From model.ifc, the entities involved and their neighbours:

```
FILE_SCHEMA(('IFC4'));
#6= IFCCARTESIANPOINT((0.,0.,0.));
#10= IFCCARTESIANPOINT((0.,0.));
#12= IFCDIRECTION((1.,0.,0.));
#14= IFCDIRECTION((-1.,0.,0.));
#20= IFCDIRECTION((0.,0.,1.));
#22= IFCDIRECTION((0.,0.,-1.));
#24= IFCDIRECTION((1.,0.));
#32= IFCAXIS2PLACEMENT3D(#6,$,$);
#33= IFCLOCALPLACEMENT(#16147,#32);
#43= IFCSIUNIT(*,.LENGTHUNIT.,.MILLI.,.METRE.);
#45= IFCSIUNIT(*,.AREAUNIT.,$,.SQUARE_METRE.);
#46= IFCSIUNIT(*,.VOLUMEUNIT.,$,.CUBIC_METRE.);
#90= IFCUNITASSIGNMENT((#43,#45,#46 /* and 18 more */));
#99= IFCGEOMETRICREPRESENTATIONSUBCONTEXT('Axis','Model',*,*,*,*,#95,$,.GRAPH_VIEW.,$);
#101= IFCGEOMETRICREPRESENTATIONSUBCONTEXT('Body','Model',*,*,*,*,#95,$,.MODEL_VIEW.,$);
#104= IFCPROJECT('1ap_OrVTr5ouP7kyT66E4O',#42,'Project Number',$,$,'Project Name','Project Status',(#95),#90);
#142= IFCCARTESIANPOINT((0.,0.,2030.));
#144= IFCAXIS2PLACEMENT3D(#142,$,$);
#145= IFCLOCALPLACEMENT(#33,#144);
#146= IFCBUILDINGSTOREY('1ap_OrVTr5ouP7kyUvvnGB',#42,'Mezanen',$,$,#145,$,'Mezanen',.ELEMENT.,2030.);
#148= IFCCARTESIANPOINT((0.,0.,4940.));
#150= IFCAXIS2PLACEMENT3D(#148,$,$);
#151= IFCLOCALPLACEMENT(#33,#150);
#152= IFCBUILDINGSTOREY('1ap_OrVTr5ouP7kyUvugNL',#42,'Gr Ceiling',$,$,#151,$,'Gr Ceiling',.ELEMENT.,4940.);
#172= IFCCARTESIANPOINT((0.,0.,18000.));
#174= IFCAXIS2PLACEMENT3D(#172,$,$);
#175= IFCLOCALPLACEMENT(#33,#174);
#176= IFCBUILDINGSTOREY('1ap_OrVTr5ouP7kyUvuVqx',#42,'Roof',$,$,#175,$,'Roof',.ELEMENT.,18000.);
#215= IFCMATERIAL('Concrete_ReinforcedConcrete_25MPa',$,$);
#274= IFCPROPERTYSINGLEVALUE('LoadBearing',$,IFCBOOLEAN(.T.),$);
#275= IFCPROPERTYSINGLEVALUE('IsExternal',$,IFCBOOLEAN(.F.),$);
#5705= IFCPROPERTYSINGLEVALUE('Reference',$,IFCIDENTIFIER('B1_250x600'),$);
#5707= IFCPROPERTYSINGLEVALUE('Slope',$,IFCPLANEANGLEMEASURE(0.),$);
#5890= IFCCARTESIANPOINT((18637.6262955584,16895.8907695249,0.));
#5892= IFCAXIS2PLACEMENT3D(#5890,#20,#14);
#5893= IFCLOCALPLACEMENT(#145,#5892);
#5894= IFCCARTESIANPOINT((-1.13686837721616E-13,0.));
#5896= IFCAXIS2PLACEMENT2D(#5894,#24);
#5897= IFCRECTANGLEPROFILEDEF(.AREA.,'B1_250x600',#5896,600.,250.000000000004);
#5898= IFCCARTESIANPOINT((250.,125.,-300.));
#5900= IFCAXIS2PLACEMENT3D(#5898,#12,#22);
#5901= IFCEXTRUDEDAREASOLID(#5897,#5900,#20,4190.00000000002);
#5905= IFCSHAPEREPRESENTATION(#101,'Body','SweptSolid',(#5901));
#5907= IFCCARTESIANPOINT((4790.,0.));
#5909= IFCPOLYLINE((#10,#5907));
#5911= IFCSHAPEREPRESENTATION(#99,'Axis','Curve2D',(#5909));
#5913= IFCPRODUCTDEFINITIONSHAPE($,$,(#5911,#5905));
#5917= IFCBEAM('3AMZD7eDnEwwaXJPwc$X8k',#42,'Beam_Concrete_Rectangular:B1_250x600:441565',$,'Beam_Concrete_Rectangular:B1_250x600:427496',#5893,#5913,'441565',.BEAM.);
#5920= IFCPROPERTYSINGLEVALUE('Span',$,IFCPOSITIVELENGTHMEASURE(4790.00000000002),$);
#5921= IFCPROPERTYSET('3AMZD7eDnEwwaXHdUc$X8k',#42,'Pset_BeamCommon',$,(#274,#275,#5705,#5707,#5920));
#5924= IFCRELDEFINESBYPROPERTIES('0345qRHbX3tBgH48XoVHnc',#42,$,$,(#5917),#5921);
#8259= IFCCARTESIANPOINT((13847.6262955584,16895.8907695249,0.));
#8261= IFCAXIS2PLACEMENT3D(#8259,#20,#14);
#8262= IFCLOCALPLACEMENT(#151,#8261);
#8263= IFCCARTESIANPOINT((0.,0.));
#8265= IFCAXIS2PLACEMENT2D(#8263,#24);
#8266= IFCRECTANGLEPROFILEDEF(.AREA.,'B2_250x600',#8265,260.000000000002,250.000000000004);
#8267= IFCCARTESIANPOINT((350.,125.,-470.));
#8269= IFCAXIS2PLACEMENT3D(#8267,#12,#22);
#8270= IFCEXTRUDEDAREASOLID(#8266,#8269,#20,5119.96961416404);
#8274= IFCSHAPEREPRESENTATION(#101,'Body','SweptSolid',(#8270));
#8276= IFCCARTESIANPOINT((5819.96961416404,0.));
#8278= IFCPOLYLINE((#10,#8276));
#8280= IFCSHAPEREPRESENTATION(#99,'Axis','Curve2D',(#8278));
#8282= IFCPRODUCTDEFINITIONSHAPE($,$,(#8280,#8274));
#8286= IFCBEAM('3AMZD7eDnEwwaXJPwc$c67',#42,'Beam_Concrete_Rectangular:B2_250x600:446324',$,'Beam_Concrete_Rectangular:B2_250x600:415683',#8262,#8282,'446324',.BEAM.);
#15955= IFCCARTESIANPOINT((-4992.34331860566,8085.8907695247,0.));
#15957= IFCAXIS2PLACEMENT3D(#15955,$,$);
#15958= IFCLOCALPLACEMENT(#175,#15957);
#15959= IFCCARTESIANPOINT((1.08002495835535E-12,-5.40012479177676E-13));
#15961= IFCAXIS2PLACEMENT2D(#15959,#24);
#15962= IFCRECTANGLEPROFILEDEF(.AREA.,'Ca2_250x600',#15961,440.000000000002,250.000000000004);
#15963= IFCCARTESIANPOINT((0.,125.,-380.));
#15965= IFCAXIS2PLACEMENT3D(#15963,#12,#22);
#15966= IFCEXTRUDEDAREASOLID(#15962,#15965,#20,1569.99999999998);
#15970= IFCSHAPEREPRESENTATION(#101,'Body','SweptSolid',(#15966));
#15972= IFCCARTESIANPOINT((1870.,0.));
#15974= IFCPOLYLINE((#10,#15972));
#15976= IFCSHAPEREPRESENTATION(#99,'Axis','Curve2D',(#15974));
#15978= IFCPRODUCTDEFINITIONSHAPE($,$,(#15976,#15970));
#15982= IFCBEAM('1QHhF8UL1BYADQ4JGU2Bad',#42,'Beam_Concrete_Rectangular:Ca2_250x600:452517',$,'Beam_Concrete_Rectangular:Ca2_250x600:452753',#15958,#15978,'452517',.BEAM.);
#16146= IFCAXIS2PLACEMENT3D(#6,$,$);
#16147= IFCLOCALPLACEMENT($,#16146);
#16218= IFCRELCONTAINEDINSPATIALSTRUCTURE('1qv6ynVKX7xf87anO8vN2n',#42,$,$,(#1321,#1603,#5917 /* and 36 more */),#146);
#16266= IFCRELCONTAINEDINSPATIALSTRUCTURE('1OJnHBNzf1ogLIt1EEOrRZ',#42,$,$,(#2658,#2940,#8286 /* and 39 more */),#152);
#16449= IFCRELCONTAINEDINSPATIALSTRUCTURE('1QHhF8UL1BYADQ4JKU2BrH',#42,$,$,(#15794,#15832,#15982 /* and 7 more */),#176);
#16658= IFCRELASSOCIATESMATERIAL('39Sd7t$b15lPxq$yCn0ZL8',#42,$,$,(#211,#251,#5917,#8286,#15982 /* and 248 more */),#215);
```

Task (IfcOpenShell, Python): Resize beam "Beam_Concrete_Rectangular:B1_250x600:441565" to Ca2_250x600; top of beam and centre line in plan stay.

```python
import ifcopenshell
import ifcopenshell.api.pset
import ifcopenshell.util.element
import ifcopenshell.util.representation

model = ifcopenshell.open("model.ifc")

member = model.by_guid("3AMZD7eDnEwwaXJPwc$X8k")
source = next(p for p in model.by_type("IfcRectangleProfileDef") if p.ProfileName == "Ca2_250x600")

body = ifcopenshell.util.representation.get_representation(member, "Model", "Body")
solid = body.Items[0]
old_profile = solid.SweptArea

# Copy the section's sizes but keep this member's own profile position.
profile = ifcopenshell.util.element.copy(model, source)
# Profiles are centred, so shift by half the change in depth to hold the top.
shift = (old_profile.XDim - profile.XDim) / 2
x, y = old_profile.Position.Location.Coordinates
up = (-1.0, 0.0)  # upwards, in the solid's own plane
location = model.createIfcCartesianPoint((x + up[0] * shift, y + up[1] * shift))
profile.Position = model.createIfcAxis2Placement2D(location, old_profile.Position.RefDirection)
solid.SweptArea = profile
if not model.get_total_inverses(old_profile):
    ifcopenshell.util.element.remove_deep2(model, old_profile)
member.Name = member.Name.replace("B1_250x600", "Ca2_250x600")
member.ObjectType = member.ObjectType.replace("B1_250x600", "Ca2_250x600")
pset = model.by_id(ifcopenshell.util.element.get_pset(member, "Pset_BeamCommon", should_inherit=False)["id"])
ifcopenshell.api.pset.edit_pset(model, pset=pset, properties={"Reference": "Ca2_250x600"})

print(solid.SweptArea)

model.write("model_edited.ifc")
```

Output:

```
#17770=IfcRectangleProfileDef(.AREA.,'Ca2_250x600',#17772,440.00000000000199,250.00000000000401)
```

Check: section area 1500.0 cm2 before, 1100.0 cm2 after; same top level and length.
